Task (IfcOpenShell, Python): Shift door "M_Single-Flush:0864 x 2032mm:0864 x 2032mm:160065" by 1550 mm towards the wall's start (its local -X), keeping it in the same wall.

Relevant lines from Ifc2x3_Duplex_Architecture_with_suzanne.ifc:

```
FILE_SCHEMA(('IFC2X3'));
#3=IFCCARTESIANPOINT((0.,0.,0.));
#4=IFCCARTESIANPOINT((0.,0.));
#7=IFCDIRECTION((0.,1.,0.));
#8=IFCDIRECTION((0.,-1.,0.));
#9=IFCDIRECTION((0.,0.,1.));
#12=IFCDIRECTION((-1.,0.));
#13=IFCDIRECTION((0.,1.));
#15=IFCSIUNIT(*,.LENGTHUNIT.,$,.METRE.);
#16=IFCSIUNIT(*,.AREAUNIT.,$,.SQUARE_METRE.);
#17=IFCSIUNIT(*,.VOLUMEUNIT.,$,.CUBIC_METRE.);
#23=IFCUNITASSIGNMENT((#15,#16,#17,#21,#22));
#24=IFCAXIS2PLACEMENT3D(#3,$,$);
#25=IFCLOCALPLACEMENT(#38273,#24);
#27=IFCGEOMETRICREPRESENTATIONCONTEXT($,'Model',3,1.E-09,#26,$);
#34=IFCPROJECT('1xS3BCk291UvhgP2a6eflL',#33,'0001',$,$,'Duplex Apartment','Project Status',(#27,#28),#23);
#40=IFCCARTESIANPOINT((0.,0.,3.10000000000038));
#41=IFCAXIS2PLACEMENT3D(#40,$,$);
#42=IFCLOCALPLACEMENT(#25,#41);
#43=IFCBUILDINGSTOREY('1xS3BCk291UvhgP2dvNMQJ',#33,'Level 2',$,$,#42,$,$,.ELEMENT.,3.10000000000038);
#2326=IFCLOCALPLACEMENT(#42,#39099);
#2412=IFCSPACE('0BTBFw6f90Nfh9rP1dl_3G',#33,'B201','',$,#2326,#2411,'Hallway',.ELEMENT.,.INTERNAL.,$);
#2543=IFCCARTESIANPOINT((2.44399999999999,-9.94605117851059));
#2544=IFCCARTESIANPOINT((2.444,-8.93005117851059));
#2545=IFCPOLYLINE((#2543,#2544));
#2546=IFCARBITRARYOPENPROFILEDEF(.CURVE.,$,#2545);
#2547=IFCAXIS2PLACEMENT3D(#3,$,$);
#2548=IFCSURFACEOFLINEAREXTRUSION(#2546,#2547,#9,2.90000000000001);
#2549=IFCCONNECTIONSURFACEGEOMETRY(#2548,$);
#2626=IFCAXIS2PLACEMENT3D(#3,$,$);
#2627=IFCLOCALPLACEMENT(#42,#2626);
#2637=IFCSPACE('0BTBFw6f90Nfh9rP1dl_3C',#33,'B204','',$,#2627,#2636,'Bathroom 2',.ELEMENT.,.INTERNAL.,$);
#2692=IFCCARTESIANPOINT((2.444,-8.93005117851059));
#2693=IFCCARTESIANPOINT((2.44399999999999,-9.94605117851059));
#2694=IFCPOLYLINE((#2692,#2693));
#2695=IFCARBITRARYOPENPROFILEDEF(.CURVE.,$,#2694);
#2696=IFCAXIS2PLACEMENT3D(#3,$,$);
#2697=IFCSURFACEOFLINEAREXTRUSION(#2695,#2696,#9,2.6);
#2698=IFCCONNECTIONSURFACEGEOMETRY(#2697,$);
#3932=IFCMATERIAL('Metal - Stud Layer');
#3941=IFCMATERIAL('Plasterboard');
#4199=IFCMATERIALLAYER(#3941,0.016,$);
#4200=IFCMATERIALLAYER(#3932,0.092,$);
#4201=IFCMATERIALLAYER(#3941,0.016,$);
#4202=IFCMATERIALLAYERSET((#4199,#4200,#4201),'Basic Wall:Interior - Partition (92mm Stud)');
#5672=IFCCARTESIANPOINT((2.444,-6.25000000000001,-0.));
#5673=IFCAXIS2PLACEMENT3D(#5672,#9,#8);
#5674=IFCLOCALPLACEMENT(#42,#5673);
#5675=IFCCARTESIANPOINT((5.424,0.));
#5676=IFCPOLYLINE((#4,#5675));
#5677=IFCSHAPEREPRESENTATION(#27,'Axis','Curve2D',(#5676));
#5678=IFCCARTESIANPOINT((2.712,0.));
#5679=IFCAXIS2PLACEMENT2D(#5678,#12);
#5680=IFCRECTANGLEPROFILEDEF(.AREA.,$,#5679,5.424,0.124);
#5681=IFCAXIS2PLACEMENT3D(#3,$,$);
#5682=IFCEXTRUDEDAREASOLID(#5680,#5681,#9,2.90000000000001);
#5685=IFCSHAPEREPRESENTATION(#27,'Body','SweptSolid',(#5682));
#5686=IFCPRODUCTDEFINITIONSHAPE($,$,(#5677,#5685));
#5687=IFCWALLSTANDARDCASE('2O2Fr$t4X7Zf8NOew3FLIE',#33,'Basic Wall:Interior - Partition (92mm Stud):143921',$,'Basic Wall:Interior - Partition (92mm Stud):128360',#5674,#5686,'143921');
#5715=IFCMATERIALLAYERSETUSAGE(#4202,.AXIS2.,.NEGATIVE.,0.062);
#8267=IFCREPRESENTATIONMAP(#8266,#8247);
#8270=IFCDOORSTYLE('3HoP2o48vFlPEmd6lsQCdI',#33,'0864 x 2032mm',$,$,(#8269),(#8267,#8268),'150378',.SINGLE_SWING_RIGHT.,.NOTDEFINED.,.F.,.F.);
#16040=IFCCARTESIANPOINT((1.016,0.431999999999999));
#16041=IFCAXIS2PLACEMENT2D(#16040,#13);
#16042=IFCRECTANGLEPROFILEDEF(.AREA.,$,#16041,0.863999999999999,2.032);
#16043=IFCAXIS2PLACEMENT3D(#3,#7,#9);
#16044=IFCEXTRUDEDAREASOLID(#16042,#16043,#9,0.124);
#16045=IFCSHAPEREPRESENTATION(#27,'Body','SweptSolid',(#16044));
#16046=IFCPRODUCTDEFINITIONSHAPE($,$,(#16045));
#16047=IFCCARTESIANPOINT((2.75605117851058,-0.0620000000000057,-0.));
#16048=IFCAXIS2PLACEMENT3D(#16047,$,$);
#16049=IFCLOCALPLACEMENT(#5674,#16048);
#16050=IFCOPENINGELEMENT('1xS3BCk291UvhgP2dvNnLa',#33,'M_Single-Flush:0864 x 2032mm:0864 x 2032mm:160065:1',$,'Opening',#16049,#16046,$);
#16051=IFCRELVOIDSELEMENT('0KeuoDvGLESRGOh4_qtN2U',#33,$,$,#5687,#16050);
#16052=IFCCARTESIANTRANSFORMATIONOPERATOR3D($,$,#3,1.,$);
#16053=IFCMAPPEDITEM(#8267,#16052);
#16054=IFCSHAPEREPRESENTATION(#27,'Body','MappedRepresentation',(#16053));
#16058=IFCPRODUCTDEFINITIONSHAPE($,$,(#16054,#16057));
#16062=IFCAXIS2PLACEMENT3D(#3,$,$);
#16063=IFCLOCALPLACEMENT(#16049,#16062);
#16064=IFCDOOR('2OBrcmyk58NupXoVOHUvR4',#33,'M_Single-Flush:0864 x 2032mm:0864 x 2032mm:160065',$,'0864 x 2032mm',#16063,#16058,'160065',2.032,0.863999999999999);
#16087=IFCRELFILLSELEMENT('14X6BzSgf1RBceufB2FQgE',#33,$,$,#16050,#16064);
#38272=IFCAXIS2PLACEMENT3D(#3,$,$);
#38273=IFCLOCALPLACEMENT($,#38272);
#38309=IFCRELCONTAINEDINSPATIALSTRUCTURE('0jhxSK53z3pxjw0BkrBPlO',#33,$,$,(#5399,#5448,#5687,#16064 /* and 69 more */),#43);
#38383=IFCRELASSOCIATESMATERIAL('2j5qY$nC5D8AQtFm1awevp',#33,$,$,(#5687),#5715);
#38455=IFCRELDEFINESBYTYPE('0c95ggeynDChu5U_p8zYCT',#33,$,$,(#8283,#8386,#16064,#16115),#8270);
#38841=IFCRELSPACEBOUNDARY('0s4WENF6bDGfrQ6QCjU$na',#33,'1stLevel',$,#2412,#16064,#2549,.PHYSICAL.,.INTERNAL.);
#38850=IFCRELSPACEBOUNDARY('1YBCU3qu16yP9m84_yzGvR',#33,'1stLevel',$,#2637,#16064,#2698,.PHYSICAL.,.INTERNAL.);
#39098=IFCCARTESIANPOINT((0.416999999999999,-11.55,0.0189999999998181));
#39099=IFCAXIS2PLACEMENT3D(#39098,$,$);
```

```python
import numpy as np
import ifcopenshell
import ifcopenshell.api.geometry
import ifcopenshell.util.placement
import ifcopenshell.util.unit

model = ifcopenshell.open("Ifc2x3_Duplex_Architecture_with_suzanne.ifc")
unit_scale = ifcopenshell.util.unit.calculate_unit_scale(model)

door = model.by_guid("2OBrcmyk58NupXoVOHUvR4")
opening = door.FillsVoids[0].RelatingOpeningElement
wall = opening.VoidsElements[0].RelatingBuildingElement

wall_matrix = ifcopenshell.util.placement.get_local_placement(wall.ObjectPlacement)
shift = wall_matrix[:3, 0] * -1.55 / unit_scale
before = ifcopenshell.util.placement.get_local_placement(door.ObjectPlacement)[:3, 3].copy()

# The door is placed relative to its opening, so it follows when the opening moves.
matrix = ifcopenshell.util.placement.get_local_placement(opening.ObjectPlacement)
matrix[:3, 3] += shift
ifcopenshell.api.geometry.edit_object_placement(
    model, product=opening, matrix=matrix, is_si=False, should_transform_children=True
)

# Space boundary surfaces are stored in each space's coordinates; move them too.
for rel in door.ProvidesBoundaries:
    if not rel.ConnectionGeometry:
        continue
    surface = rel.ConnectionGeometry.SurfaceOnRelatingElement
    space_matrix = ifcopenshell.util.placement.get_local_placement(rel.RelatingSpace.ObjectPlacement)
    point = np.array(surface.Position.Location.Coordinates) + space_matrix[:3, :3].T @ shift
    surface.Position = model.createIfcAxis2Placement3D(
        model.createIfcCartesianPoint(point.tolist()), surface.Position.Axis, surface.Position.RefDirection
    )

after = ifcopenshell.util.placement.get_local_placement(door.ObjectPlacement)[:3, 3]
print("door moved by", (after - before).round(3) + 0.0)

model.write("Ifc2x3_Duplex_Architecture_with_suzanne_v2.ifc")
```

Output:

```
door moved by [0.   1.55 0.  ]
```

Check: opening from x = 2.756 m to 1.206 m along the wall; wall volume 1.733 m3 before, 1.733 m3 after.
